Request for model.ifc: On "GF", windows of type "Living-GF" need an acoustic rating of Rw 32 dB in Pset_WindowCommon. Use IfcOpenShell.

First a look at what the model holds.

```python
import ifcopenshell
import ifcopenshell.util.element

model = ifcopenshell.open("model.ifc")
print(model.schema)
storey = next(s for s in model.by_type("IfcBuildingStorey") if s.Name == "GF")
windows = [e for e in ifcopenshell.util.element.get_decomposition(storey) if e.is_a("IfcWindow")]
seen = {}
for e in windows:
    element_type = ifcopenshell.util.element.get_type(e)
    key = (element_type.Name if element_type != e and element_type else None, ifcopenshell.util.element.get_pset(e, "Pset_WindowCommon", "AcousticRating"))
    seen[key] = seen.get(key, 0) + 1
for (name, value), count in sorted(seen.items(), key=str):
    print(count, "x", name, "|", value)
```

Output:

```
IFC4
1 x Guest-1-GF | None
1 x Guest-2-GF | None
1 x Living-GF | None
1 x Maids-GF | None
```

```python
import ifcopenshell
import ifcopenshell.api.pset
import ifcopenshell.util.element

model = ifcopenshell.open("model.ifc")

storey = next(s for s in model.by_type("IfcBuildingStorey") if s.Name == "GF")
windows = [e for e in ifcopenshell.util.element.get_decomposition(storey) if e.is_a("IfcWindow")]

count = 0
for e in windows:
    element_type = ifcopenshell.util.element.get_type(e)
    if element_type in (None, e) or element_type.Name != "Living-GF":
        continue
    # add_pset returns the element's existing set when there is one.
    pset = ifcopenshell.api.pset.add_pset(model, product=e, name="Pset_WindowCommon")
    ifcopenshell.api.pset.edit_pset(model, pset=pset, properties={"AcousticRating": "Rw 32 dB"})
    count += 1

print(count, "windows updated")

model.write("model_v2.ifc")
```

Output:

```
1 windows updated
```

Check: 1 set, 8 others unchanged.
